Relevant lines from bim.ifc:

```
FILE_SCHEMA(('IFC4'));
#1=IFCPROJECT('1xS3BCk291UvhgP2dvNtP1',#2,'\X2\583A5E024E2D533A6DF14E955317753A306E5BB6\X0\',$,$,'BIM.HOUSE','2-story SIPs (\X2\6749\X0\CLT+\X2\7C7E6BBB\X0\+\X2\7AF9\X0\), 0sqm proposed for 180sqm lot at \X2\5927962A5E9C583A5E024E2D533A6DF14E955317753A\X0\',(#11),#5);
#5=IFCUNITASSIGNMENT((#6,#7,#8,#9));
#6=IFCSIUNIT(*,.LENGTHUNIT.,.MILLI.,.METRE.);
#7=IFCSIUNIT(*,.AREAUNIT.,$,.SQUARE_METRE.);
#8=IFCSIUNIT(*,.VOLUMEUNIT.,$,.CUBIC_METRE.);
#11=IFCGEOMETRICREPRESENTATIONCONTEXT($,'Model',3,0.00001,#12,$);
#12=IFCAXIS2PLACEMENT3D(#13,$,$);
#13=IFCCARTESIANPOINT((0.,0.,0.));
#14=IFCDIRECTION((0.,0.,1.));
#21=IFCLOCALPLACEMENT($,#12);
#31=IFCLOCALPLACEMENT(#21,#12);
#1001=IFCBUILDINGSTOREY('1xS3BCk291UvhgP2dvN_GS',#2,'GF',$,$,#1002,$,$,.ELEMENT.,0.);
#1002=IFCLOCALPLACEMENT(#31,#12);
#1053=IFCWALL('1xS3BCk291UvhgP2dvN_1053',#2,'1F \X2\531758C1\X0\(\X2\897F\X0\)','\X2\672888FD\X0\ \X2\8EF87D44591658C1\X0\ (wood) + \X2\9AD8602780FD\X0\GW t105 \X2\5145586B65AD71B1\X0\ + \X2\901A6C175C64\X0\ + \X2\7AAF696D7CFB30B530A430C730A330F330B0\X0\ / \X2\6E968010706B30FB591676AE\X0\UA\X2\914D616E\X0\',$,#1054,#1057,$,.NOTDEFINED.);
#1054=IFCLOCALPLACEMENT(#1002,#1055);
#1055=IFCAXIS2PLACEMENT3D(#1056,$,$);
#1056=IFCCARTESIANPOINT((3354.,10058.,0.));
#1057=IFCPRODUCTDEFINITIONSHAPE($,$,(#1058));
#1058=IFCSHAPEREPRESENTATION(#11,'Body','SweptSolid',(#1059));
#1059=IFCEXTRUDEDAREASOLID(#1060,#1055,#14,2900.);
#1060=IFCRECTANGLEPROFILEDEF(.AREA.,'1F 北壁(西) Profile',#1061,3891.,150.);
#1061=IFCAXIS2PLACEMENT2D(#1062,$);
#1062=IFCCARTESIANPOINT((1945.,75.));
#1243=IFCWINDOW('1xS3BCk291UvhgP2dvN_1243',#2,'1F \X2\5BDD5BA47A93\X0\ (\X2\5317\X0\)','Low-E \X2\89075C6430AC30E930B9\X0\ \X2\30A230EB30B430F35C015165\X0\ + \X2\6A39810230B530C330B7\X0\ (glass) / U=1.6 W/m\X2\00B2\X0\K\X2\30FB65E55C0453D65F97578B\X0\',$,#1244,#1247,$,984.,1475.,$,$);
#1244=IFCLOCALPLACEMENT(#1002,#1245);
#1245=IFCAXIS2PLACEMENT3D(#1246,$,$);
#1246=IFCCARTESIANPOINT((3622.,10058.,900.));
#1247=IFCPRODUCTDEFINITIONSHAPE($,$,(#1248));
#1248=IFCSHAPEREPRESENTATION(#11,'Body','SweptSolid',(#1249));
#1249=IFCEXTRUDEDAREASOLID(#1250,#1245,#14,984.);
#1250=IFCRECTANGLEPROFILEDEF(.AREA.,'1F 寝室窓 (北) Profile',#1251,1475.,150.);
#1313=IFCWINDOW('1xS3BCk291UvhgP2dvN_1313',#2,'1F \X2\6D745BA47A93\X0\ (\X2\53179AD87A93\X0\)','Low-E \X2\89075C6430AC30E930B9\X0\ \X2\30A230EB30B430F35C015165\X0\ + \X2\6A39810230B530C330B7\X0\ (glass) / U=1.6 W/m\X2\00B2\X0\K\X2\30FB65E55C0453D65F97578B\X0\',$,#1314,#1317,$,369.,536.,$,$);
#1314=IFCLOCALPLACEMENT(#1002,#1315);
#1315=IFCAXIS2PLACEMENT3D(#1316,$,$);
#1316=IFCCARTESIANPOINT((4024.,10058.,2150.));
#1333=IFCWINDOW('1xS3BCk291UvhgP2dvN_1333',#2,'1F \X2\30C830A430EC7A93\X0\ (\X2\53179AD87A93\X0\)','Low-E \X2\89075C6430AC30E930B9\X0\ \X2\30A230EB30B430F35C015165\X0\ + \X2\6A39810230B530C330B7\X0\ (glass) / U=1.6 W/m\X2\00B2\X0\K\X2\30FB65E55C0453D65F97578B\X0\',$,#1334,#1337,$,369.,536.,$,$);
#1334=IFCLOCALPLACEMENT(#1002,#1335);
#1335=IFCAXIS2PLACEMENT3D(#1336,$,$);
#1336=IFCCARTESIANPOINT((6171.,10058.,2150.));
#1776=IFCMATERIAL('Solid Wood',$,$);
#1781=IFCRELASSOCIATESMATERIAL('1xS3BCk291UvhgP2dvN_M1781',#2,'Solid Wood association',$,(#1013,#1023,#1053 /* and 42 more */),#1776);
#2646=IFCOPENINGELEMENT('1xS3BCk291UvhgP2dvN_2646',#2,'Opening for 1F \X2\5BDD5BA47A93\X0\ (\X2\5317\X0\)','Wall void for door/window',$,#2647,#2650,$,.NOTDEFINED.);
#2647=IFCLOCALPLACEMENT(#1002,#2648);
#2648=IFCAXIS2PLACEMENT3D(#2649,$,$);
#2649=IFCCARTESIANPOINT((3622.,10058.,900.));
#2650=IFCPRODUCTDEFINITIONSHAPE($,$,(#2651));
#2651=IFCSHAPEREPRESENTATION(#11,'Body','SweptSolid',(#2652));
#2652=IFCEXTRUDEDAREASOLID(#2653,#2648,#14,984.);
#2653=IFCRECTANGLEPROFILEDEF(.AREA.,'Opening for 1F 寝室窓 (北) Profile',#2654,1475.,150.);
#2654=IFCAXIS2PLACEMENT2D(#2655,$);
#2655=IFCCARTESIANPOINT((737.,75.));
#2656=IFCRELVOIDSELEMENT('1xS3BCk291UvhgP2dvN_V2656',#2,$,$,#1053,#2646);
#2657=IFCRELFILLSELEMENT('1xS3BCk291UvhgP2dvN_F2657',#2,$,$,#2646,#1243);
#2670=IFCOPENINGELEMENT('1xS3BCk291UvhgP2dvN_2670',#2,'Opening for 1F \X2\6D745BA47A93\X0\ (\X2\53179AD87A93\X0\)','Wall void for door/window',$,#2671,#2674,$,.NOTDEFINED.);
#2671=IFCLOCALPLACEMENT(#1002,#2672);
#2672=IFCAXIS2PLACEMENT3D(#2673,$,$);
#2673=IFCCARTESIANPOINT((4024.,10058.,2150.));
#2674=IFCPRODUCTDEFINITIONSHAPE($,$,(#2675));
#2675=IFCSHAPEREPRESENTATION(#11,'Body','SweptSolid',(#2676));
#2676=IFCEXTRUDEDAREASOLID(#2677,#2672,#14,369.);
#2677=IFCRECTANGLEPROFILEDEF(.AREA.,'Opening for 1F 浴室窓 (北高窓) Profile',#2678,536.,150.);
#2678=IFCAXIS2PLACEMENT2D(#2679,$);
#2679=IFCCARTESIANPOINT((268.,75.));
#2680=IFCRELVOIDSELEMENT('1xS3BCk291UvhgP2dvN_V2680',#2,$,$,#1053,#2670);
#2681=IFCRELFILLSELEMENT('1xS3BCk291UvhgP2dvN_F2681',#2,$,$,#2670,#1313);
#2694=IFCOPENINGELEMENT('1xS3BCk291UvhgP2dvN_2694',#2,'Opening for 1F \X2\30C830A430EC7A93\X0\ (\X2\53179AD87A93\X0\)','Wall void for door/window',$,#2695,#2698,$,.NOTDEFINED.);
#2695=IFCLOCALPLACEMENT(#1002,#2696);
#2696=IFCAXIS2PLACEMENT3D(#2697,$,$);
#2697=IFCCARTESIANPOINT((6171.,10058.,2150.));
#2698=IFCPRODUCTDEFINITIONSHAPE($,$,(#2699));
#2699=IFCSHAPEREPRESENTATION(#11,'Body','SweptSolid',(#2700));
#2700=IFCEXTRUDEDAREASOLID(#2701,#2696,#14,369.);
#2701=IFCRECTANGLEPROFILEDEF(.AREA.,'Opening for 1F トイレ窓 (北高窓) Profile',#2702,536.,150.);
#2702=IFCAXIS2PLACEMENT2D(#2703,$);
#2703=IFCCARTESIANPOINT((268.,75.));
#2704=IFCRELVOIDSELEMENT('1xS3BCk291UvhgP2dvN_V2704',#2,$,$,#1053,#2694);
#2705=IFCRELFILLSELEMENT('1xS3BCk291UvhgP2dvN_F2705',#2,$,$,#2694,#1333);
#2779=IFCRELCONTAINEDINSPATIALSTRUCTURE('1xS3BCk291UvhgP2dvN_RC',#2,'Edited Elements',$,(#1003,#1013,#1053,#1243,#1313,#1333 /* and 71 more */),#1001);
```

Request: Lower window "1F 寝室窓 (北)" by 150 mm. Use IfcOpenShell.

```python
import numpy as np
import ifcopenshell
import ifcopenshell.api.geometry
import ifcopenshell.util.placement
import ifcopenshell.util.unit

model = ifcopenshell.open("bim.ifc")
unit_scale = ifcopenshell.util.unit.calculate_unit_scale(model)

window = model.by_guid("1xS3BCk291UvhgP2dvN_1243")
opening = window.FillsVoids[0].RelatingOpeningElement
dz = -0.15 / unit_scale

shift = np.array([0.0, 0.0, dz])
# The window is not placed relative to its opening, so move both.
for product in (opening, window):
    matrix = ifcopenshell.util.placement.get_local_placement(product.ObjectPlacement)
    matrix[:3, 3] += shift
    ifcopenshell.api.geometry.edit_object_placement(model, product=product, matrix=matrix, is_si=False)

print(f"moved by {dz * unit_scale:+.3f} m")

model.write("bim_edited.ifc")
```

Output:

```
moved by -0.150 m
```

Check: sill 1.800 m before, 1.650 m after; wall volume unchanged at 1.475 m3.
